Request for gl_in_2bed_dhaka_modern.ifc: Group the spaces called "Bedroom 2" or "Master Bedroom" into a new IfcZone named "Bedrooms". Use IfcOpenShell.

First a look at what the model holds.

```python
import ifcopenshell

model = ifcopenshell.open("gl_in_2bed_dhaka_modern.ifc")
print(model.schema)
seen = {}
for space in model.by_type("IfcSpace"):
    seen[space.LongName] = seen.get(space.LongName, 0) + 1
for name, count in sorted(seen.items(), key=str):
    print(count, "x", name)
print("zones:", [z.Name for z in model.by_type("IfcZone")][:20])
```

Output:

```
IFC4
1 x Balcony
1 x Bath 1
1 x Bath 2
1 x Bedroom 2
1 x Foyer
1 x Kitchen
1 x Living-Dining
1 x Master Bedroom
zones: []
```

```python
import ifcopenshell
import ifcopenshell.api.group
import ifcopenshell.api.root

model = ifcopenshell.open("gl_in_2bed_dhaka_modern.ifc")

names = {"Bedroom 2", "Master Bedroom"}
spaces = [s for s in model.by_type("IfcSpace") if s.LongName in names]

zone = ifcopenshell.api.root.create_entity(model, ifc_class="IfcZone", name="Bedrooms")
ifcopenshell.api.group.assign_group(model, products=spaces, group=zone)
print(len(spaces), "spaces in", zone.Name)

model.write("gl_in_2bed_dhaka_modern_v2.ifc")
```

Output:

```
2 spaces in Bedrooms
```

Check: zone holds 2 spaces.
